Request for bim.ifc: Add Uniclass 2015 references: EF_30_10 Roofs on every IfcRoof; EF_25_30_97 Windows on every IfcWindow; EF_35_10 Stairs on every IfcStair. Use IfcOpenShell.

First a look at what the model holds.

```python
import ifcopenshell

model = ifcopenshell.open("bim.ifc")
print(model.schema)
print("classifications:", [c.Name for c in model.by_type("IfcClassification")])
for ifc_class in ("IfcDoor", "IfcRoof", "IfcStair", "IfcWall", "IfcWindow"):
    print(ifc_class, len(model.by_type(ifc_class)))
```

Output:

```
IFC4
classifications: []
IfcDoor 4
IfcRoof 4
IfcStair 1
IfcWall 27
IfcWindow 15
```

```python
import ifcopenshell
import ifcopenshell.api.classification

model = ifcopenshell.open("bim.ifc")

system = ifcopenshell.api.classification.add_classification(model, classification="Uniclass 2015")

codes = {
    "IfcRoof": ("EF_30_10", "Roofs"),
    "IfcWindow": ("EF_25_30_97", "Windows"),
    "IfcStair": ("EF_35_10", "Stairs"),
}
for ifc_class, (code, name) in codes.items():
    products = model.by_type(ifc_class)
    ifcopenshell.api.classification.add_reference(
        model, products=products, classification=system, identification=code, name=name
    )
    print(code, len(products))

model.write("bim_v2.ifc")
```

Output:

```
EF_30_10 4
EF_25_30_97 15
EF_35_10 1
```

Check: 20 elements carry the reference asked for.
